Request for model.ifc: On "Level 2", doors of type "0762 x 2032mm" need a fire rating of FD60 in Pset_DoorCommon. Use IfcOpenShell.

First a look at what the model holds.

```python
import ifcopenshell
import ifcopenshell.util.element

model = ifcopenshell.open("model.ifc")
print(model.schema)
storey = next(s for s in model.by_type("IfcBuildingStorey") if s.Name == "Level 2")
doors = [e for e in ifcopenshell.util.element.get_decomposition(storey) if e.is_a("IfcDoor")]
seen = {}
for e in doors:
    element_type = ifcopenshell.util.element.get_type(e)
    key = (element_type.Name if element_type != e and element_type else None, ifcopenshell.util.element.get_pset(e, "Pset_DoorCommon", "FireRating"))
    seen[key] = seen.get(key, 0) + 1
for (name, value), count in sorted(seen.items(), key=str):
    print(count, "x", name, "|", value)
```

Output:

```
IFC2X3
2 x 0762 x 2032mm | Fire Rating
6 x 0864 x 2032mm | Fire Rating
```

```python
import ifcopenshell
import ifcopenshell.api.pset
import ifcopenshell.util.element

model = ifcopenshell.open("model.ifc")

storey = next(s for s in model.by_type("IfcBuildingStorey") if s.Name == "Level 2")
doors = [e for e in ifcopenshell.util.element.get_decomposition(storey) if e.is_a("IfcDoor")]

count = 0
for e in doors:
    element_type = ifcopenshell.util.element.get_type(e)
    if element_type in (None, e) or element_type.Name != "0762 x 2032mm":
        continue
    # add_pset returns the element's existing set when there is one.
    pset = ifcopenshell.api.pset.add_pset(model, product=e, name="Pset_DoorCommon")
    ifcopenshell.api.pset.edit_pset(model, pset=pset, properties={"FireRating": "FD60"})
    count += 1

print(count, "doors updated")

model.write("model-out.ifc")
```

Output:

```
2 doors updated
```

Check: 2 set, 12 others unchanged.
